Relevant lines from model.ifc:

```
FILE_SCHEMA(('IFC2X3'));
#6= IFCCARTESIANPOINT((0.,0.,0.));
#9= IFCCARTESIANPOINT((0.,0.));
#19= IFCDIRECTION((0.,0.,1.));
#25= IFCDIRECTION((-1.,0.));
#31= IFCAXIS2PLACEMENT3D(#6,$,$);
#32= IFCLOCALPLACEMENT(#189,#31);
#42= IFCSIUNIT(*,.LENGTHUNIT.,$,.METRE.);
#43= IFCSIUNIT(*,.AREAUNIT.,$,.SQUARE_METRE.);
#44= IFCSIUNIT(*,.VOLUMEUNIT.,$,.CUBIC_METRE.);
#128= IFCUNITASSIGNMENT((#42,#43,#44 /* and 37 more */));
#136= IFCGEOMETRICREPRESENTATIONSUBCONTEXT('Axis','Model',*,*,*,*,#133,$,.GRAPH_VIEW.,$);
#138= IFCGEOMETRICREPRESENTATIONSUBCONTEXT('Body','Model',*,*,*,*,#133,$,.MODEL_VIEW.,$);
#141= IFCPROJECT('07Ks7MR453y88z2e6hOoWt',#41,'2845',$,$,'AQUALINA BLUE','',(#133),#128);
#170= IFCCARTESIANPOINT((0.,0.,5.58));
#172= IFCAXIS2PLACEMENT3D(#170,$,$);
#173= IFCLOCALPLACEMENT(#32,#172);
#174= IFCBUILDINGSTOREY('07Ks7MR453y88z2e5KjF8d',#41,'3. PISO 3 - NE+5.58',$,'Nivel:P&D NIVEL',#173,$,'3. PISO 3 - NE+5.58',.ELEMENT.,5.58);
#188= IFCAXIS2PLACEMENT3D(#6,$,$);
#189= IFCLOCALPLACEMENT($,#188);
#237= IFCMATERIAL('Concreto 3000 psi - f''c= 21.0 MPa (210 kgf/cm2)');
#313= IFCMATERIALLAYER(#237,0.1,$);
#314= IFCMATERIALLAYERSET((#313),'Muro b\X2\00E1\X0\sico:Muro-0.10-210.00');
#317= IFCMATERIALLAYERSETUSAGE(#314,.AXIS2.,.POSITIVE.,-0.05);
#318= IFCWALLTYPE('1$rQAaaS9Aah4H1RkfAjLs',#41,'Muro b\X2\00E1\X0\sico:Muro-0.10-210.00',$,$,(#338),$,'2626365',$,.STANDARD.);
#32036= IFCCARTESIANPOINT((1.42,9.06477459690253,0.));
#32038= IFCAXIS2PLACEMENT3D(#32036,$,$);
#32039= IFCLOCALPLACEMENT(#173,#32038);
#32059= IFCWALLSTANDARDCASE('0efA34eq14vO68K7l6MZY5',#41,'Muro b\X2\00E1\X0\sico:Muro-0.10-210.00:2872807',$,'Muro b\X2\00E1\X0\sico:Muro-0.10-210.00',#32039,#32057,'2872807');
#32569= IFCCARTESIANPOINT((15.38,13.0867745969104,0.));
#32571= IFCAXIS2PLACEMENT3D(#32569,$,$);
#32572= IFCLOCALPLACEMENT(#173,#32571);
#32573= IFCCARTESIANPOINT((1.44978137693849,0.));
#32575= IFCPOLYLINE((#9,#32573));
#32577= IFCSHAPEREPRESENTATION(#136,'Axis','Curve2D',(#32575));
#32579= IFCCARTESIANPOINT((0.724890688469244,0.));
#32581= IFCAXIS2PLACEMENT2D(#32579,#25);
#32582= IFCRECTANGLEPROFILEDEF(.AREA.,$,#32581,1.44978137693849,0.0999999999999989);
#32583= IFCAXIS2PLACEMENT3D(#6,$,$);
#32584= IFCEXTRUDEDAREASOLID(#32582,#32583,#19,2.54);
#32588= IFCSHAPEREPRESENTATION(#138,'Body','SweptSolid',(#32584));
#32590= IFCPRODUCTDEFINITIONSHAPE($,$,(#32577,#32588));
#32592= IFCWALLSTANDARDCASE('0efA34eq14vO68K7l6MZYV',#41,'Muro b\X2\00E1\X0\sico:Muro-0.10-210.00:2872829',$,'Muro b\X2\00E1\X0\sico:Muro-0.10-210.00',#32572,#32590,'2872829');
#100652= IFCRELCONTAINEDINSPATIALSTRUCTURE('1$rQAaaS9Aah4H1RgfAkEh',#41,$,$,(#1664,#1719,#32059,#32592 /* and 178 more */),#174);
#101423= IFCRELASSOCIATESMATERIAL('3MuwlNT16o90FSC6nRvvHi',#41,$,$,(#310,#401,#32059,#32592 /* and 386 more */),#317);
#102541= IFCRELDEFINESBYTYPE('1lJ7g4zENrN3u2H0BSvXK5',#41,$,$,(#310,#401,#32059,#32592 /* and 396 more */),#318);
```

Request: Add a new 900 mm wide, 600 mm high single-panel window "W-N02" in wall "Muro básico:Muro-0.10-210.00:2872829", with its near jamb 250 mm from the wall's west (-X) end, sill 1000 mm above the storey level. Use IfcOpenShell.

```python
import numpy as np
import ifcopenshell
import ifcopenshell.api.feature
import ifcopenshell.api.geometry
import ifcopenshell.api.root
import ifcopenshell.api.spatial
import ifcopenshell.api.type
import ifcopenshell.geom
import ifcopenshell.util.element
import ifcopenshell.util.placement
import ifcopenshell.util.representation
import ifcopenshell.util.shape
import ifcopenshell.util.unit

model = ifcopenshell.open("model.ifc")
unit_scale = ifcopenshell.util.unit.calculate_unit_scale(model)
settings = ifcopenshell.geom.settings()


def volume(element):
    """Net volume in cubic metres, openings subtracted."""
    shape = ifcopenshell.geom.create_shape(settings, element)
    return ifcopenshell.util.shape.get_volume(shape.geometry)


wall = model.by_guid("0efA34eq14vO68K7l6MZYV")
storey = ifcopenshell.util.element.get_container(wall, ifc_class="IfcBuildingStorey")
context = ifcopenshell.util.representation.get_context(model, "Model", "Body", "MODEL_VIEW")
before = volume(wall)

width, height, from_end, sill = 0.9, 0.6, 0.25, 1  # metres

# The wall runs along its own X axis, and the end named is its -X end.
wall_shape = ifcopenshell.geom.create_shape(settings, wall)
x, y, z = ifcopenshell.util.shape.get_vertices(wall_shape.geometry).T
start = x.min() + from_end
face, thickness = float(y.min()), float(y.max() - y.min())
wall_matrix = ifcopenshell.util.placement.get_local_placement(wall.ObjectPlacement)
level = ifcopenshell.util.placement.get_local_placement(storey.ObjectPlacement)[2, 3]


def in_wall(x, y):
    """Placement at x, y metres in the wall's axes, at sill height."""
    matrix = wall_matrix.copy()
    matrix[:, 3] = wall_matrix @ np.array([x / unit_scale, y / unit_scale, 0.0, 1.0])
    matrix[2, 3] = level + sill / unit_scale
    return matrix


# Opening: a box that overshoots both wall faces by 50 mm.
opening = ifcopenshell.api.root.create_entity(model, ifc_class="IfcOpeningElement")
box = ifcopenshell.api.geometry.add_wall_representation(
    model, context=context, length=width, height=height, thickness=thickness + 0.1
)
ifcopenshell.api.geometry.assign_representation(model, product=opening, representation=box)
ifcopenshell.api.geometry.edit_object_placement(model, product=opening, matrix=in_wall(start, face - 0.05), is_si=False)
ifcopenshell.api.feature.add_feature(model, feature=opening, element=wall)

window = ifcopenshell.api.root.create_entity(model, ifc_class="IfcWindow", name="W-N02")
window.OverallWidth, window.OverallHeight = width / unit_scale, height / unit_scale
body = ifcopenshell.api.geometry.add_window_representation(
    model,
    context=context,
    overall_width=window.OverallWidth,
    overall_height=window.OverallHeight,
    partition_type="SINGLE_PANEL",
)
ifcopenshell.api.geometry.assign_representation(model, product=window, representation=body)
ifcopenshell.api.spatial.assign_container(model, products=[window], relating_structure=storey)
fills = ifcopenshell.api.feature.add_filling(model, opening=opening, element=window)
fills.OwnerHistory = window.OwnerHistory  # required in IFC2X3

# IFC2X3 keeps the operation on the window style.
style = ifcopenshell.api.root.create_entity(model, ifc_class="IfcWindowStyle", name="W-N02")
style.OperationType, style.ConstructionType = "SINGLE_PANEL", "NOTDEFINED"
style.ParameterTakesPrecedence = style.Sizeable = False
ifcopenshell.api.type.assign_type(model, related_objects=[window], relating_type=style)

# Centre the window in the wall's thickness.
ifcopenshell.api.geometry.edit_object_placement(model, product=window, matrix=in_wall(start, face), is_si=False)
window_shape = ifcopenshell.geom.create_shape(settings, window)
depth = ifcopenshell.util.shape.get_vertices(window_shape.geometry)[:, 1]
offset = face + thickness / 2 - (depth.min() + depth.max()) / 2
ifcopenshell.api.geometry.edit_object_placement(model, product=window, matrix=in_wall(start, offset), is_si=False)

after = volume(wall)

print(f"wall volume {before:.3f} -> {after:.3f} m3")

model.write("model-out.ifc")
```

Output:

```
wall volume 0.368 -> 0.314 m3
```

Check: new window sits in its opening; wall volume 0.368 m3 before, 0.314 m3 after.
